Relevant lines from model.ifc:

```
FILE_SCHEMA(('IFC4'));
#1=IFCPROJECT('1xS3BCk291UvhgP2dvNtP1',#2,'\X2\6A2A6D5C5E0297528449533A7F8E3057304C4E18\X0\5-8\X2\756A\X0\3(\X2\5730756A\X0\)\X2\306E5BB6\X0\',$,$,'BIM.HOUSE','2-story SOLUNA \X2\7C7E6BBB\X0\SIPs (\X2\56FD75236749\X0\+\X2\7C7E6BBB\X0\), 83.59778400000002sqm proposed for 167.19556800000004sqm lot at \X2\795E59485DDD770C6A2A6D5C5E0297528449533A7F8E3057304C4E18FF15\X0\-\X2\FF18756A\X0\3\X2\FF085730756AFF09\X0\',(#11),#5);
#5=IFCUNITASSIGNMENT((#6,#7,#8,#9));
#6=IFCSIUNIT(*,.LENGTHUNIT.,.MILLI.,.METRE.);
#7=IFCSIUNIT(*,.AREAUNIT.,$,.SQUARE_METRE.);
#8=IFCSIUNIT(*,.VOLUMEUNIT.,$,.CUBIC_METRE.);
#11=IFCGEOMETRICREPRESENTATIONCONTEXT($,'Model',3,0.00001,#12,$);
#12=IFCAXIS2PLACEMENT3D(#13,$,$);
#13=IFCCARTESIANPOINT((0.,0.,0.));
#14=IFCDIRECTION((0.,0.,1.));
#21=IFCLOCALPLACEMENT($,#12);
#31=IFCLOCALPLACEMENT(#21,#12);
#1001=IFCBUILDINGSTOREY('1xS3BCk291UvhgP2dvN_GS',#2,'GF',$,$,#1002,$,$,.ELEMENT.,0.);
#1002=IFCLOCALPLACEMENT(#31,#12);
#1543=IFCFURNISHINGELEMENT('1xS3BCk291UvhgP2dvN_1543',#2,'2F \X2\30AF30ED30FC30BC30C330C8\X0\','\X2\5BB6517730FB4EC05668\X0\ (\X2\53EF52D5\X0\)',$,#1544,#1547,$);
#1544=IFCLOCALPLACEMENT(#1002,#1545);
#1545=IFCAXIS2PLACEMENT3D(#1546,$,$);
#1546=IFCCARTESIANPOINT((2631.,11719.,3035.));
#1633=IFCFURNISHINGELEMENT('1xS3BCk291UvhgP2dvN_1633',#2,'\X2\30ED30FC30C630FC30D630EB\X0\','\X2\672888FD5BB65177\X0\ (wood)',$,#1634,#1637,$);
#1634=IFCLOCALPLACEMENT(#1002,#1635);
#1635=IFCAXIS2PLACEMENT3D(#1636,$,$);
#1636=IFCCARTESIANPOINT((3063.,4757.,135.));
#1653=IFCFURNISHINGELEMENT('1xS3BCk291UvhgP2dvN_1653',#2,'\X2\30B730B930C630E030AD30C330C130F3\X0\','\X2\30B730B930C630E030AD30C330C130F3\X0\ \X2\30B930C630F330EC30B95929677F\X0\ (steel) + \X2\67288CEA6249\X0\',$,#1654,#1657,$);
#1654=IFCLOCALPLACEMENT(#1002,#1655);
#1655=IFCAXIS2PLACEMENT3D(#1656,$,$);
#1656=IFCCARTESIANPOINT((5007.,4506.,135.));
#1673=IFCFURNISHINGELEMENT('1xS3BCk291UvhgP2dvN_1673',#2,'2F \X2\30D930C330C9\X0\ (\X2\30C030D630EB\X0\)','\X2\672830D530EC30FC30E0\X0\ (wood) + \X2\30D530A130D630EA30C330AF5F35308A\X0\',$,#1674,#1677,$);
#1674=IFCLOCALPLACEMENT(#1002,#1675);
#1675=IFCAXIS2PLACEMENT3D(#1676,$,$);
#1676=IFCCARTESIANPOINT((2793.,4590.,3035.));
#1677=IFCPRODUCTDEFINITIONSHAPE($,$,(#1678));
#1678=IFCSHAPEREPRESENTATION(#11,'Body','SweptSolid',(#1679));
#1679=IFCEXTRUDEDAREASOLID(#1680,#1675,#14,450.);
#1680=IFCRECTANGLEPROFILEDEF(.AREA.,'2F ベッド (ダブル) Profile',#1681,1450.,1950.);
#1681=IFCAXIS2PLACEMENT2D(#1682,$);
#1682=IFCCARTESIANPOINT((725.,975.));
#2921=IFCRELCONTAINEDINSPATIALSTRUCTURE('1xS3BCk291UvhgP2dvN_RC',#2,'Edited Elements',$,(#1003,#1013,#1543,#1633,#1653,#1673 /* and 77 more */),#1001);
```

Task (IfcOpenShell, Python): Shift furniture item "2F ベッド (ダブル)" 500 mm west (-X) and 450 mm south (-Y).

```python
import ifcopenshell
import ifcopenshell.api.geometry
import ifcopenshell.util.placement
import ifcopenshell.util.unit

model = ifcopenshell.open("model.ifc")
unit_scale = ifcopenshell.util.unit.calculate_unit_scale(model)

item = model.by_guid("1xS3BCk291UvhgP2dvN_1673")
matrix = ifcopenshell.util.placement.get_local_placement(item.ObjectPlacement)
matrix[0, 3] -= 0.5 / unit_scale
matrix[1, 3] -= 0.45 / unit_scale
ifcopenshell.api.geometry.edit_object_placement(model, product=item, matrix=matrix, is_si=False)

print(ifcopenshell.util.placement.get_local_placement(item.ObjectPlacement).round(3) + 0.0)

model.write("model_rev.ifc")
```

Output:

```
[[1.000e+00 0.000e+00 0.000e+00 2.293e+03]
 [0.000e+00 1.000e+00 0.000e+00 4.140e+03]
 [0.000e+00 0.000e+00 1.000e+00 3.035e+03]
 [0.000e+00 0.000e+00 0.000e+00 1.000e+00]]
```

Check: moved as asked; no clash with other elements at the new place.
